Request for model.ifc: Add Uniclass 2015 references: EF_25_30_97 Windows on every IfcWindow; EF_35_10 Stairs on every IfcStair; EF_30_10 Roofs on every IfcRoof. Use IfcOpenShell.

First a look at what the model holds.

```python
import ifcopenshell

model = ifcopenshell.open("model.ifc")
print(model.schema)
print("classifications:", [c.Name for c in model.by_type("IfcClassification")])
for ifc_class in ("IfcDoor", "IfcRoof", "IfcStair", "IfcWall", "IfcWindow"):
    print(ifc_class, len(model.by_type(ifc_class)))
```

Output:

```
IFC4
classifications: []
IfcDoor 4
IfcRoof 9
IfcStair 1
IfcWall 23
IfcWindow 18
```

```python
import ifcopenshell
import ifcopenshell.api.classification

model = ifcopenshell.open("model.ifc")

system = ifcopenshell.api.classification.add_classification(model, classification="Uniclass 2015")

codes = {
    "IfcWindow": ("EF_25_30_97", "Windows"),
    "IfcStair": ("EF_35_10", "Stairs"),
    "IfcRoof": ("EF_30_10", "Roofs"),
}
for ifc_class, (code, name) in codes.items():
    products = model.by_type(ifc_class)
    ifcopenshell.api.classification.add_reference(
        model, products=products, classification=system, identification=code, name=name
    )
    print(code, len(products))

model.write("model-out.ifc")
```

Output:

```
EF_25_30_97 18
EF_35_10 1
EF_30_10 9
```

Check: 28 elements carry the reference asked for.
